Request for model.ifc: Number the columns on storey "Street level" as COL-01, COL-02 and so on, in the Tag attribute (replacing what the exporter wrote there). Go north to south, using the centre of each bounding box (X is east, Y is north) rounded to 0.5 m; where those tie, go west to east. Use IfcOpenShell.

First a look at what the model holds.

```python
import ifcopenshell
import ifcopenshell.util.element
import ifcopenshell.util.placement

model = ifcopenshell.open("model.ifc")
print(model.schema)
storey = next(s for s in model.by_type("IfcBuildingStorey") if s.Name == "Street level")
columns = [e for e in ifcopenshell.util.element.get_decomposition(storey) if e.is_a("IfcColumn")]
for e in sorted(columns, key=lambda e: e.id()):
    origin = ifcopenshell.util.placement.get_local_placement(e.ObjectPlacement)[:3, 3]
    print(e.id(), e.Tag, e.Name, origin.round(2) + 0.0, sep=" | ")
```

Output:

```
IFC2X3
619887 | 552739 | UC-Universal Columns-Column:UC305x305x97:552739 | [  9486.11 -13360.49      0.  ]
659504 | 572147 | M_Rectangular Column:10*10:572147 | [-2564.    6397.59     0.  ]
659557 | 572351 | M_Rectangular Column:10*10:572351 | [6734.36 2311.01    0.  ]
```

```python
import ifcopenshell
import ifcopenshell.geom
import ifcopenshell.util.element
import ifcopenshell.util.shape

model = ifcopenshell.open("model.ifc")
settings = ifcopenshell.geom.settings()
settings.set("use-world-coords", True)


def centre(element):
    shape = ifcopenshell.geom.create_shape(settings, element)
    return ifcopenshell.util.shape.get_bbox_centroid(shape.geometry)


storey = next(s for s in model.by_type("IfcBuildingStorey") if s.Name == "Street level")
columns = [e for e in ifcopenshell.util.element.get_decomposition(storey) if e.is_a("IfcColumn")]

# Insertion points can sit at a corner or the storey origin, so sort by the geometry (in metres).
centres = {e: centre(e) for e in columns}
columns.sort(key=lambda e: (-round(centres[e][1] / 0.5), centres[e][0]))

for i, e in enumerate(columns, start=1):
    number = f"COL-{i:02d}"
    e.Tag = number
    print(e.id(), number)

model.write("model_rev.ifc")
```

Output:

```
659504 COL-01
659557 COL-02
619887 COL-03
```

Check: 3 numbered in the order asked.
